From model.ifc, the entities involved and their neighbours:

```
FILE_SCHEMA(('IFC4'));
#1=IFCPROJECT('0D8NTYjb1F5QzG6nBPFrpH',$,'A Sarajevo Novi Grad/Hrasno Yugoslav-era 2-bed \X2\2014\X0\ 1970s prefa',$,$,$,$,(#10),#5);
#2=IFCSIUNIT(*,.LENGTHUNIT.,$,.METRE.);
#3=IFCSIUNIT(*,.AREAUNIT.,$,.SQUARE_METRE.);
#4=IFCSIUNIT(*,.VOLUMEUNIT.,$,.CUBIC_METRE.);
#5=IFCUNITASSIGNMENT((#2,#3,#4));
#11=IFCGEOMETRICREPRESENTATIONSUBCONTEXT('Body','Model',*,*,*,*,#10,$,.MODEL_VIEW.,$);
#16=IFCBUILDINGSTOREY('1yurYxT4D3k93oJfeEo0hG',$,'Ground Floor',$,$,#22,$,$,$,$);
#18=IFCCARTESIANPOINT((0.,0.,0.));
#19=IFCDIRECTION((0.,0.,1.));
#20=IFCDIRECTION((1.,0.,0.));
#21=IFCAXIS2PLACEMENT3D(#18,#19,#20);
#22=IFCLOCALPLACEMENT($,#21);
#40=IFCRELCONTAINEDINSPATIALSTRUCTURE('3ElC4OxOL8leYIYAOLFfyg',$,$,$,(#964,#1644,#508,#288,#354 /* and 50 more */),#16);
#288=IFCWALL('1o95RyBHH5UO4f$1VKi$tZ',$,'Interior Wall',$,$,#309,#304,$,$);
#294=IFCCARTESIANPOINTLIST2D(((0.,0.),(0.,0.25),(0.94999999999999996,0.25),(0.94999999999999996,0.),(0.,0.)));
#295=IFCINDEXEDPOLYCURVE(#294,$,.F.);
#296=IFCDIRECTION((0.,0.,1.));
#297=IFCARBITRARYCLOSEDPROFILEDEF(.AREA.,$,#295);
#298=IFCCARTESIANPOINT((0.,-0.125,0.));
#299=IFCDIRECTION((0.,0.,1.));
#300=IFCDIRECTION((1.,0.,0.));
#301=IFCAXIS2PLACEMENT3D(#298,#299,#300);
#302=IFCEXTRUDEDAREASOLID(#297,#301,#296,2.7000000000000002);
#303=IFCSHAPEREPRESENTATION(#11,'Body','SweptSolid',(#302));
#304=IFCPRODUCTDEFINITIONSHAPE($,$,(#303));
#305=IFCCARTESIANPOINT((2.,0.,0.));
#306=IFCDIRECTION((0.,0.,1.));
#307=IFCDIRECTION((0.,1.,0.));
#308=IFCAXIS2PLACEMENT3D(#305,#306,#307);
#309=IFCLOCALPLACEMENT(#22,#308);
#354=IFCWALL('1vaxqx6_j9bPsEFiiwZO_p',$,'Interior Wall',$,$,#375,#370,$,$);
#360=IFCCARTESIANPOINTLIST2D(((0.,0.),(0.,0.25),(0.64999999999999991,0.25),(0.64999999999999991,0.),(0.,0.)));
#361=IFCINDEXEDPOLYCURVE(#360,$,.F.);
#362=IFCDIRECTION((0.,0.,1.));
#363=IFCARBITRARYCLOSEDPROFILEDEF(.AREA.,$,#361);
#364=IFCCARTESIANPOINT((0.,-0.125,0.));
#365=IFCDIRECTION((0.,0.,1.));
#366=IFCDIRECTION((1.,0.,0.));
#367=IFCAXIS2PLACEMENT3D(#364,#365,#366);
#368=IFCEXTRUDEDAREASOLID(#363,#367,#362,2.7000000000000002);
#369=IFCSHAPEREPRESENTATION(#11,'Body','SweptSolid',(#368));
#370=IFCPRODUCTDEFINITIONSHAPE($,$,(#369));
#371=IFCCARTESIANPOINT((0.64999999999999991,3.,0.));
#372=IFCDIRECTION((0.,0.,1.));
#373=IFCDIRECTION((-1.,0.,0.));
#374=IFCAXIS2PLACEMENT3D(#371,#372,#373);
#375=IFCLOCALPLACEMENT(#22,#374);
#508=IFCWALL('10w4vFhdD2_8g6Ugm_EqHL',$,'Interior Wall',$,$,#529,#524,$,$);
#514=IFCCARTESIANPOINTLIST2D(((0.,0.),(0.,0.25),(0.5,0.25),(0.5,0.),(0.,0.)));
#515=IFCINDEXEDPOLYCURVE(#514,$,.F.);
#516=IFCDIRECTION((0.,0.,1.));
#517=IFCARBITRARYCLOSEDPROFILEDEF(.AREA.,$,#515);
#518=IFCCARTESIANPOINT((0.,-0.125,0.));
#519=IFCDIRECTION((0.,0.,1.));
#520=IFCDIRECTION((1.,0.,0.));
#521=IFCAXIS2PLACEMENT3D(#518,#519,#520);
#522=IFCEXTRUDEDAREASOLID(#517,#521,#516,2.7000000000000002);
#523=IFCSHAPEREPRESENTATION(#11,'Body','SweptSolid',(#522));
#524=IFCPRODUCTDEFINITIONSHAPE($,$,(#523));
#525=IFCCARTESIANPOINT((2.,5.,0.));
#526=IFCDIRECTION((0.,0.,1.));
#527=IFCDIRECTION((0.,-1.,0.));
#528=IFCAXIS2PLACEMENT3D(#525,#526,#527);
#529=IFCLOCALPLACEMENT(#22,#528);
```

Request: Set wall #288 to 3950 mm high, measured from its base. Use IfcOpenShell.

```python
import ifcopenshell
import ifcopenshell.geom
import ifcopenshell.util.representation
import ifcopenshell.util.shape
import ifcopenshell.util.unit

model = ifcopenshell.open("model.ifc")
unit_scale = ifcopenshell.util.unit.calculate_unit_scale(model)
settings = ifcopenshell.geom.settings()


def volume(element):
    """Net volume in cubic metres, openings subtracted."""
    shape = ifcopenshell.geom.create_shape(settings, element)
    return ifcopenshell.util.shape.get_volume(shape.geometry)


wall = model.by_guid("1o95RyBHH5UO4f$1VKi$tZ")
before = volume(wall)

body = ifcopenshell.util.representation.get_representation(wall, "Model", "Body")
solid = body.Items[0]
old_height = solid.Depth
solid.Depth = 3.95 / unit_scale
after = volume(wall)

print(f"height {old_height:g} -> {solid.Depth:g}, volume {before:.3f} -> {after:.3f} m3")

model.write("model-out.ifc")
```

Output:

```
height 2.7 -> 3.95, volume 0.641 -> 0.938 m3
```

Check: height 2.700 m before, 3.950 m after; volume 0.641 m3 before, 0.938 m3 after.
